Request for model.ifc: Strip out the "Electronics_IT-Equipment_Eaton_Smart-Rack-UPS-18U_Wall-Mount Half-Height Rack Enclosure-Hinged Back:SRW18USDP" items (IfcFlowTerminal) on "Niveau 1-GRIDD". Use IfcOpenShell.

First a look at what the model holds.

```python
import ifcopenshell
import ifcopenshell.util.element

model = ifcopenshell.open("model.ifc")
print(model.schema)
storey = next(s for s in model.by_type("IfcBuildingStorey") if s.Name == "Niveau 1-GRIDD")
terminals = [e for e in ifcopenshell.util.element.get_decomposition(storey) if e.is_a("IfcFlowTerminal")]
seen = {}
for e in terminals:
    element_type = ifcopenshell.util.element.get_type(e)
    name = element_type.Name if element_type not in (None, e) else None
    seen[name] = seen.get(name, 0) + 1
for name, count in sorted(seen.items(), key=str):
    print(count, "x", name)
```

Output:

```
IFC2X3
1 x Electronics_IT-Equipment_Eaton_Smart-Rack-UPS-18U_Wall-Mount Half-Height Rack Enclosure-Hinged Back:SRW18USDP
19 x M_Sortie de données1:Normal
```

```python
import ifcopenshell
import ifcopenshell.api.root
import ifcopenshell.util.element

model = ifcopenshell.open("model.ifc")

storey = next(s for s in model.by_type("IfcBuildingStorey") if s.Name == "Niveau 1-GRIDD")
terminals = [e for e in ifcopenshell.util.element.get_decomposition(storey) if e.is_a("IfcFlowTerminal")]
targets = [e for e in terminals if (t := ifcopenshell.util.element.get_type(e)) not in (None, e) and t.Name == "Electronics_IT-Equipment_Eaton_Smart-Rack-UPS-18U_Wall-Mount Half-Height Rack Enclosure-Hinged Back:SRW18USDP"]

for e in targets:
    ifcopenshell.api.root.remove_product(model, product=e)
print(len(targets), "removed")

model.write("model_rev.ifc")
```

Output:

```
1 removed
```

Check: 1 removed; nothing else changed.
